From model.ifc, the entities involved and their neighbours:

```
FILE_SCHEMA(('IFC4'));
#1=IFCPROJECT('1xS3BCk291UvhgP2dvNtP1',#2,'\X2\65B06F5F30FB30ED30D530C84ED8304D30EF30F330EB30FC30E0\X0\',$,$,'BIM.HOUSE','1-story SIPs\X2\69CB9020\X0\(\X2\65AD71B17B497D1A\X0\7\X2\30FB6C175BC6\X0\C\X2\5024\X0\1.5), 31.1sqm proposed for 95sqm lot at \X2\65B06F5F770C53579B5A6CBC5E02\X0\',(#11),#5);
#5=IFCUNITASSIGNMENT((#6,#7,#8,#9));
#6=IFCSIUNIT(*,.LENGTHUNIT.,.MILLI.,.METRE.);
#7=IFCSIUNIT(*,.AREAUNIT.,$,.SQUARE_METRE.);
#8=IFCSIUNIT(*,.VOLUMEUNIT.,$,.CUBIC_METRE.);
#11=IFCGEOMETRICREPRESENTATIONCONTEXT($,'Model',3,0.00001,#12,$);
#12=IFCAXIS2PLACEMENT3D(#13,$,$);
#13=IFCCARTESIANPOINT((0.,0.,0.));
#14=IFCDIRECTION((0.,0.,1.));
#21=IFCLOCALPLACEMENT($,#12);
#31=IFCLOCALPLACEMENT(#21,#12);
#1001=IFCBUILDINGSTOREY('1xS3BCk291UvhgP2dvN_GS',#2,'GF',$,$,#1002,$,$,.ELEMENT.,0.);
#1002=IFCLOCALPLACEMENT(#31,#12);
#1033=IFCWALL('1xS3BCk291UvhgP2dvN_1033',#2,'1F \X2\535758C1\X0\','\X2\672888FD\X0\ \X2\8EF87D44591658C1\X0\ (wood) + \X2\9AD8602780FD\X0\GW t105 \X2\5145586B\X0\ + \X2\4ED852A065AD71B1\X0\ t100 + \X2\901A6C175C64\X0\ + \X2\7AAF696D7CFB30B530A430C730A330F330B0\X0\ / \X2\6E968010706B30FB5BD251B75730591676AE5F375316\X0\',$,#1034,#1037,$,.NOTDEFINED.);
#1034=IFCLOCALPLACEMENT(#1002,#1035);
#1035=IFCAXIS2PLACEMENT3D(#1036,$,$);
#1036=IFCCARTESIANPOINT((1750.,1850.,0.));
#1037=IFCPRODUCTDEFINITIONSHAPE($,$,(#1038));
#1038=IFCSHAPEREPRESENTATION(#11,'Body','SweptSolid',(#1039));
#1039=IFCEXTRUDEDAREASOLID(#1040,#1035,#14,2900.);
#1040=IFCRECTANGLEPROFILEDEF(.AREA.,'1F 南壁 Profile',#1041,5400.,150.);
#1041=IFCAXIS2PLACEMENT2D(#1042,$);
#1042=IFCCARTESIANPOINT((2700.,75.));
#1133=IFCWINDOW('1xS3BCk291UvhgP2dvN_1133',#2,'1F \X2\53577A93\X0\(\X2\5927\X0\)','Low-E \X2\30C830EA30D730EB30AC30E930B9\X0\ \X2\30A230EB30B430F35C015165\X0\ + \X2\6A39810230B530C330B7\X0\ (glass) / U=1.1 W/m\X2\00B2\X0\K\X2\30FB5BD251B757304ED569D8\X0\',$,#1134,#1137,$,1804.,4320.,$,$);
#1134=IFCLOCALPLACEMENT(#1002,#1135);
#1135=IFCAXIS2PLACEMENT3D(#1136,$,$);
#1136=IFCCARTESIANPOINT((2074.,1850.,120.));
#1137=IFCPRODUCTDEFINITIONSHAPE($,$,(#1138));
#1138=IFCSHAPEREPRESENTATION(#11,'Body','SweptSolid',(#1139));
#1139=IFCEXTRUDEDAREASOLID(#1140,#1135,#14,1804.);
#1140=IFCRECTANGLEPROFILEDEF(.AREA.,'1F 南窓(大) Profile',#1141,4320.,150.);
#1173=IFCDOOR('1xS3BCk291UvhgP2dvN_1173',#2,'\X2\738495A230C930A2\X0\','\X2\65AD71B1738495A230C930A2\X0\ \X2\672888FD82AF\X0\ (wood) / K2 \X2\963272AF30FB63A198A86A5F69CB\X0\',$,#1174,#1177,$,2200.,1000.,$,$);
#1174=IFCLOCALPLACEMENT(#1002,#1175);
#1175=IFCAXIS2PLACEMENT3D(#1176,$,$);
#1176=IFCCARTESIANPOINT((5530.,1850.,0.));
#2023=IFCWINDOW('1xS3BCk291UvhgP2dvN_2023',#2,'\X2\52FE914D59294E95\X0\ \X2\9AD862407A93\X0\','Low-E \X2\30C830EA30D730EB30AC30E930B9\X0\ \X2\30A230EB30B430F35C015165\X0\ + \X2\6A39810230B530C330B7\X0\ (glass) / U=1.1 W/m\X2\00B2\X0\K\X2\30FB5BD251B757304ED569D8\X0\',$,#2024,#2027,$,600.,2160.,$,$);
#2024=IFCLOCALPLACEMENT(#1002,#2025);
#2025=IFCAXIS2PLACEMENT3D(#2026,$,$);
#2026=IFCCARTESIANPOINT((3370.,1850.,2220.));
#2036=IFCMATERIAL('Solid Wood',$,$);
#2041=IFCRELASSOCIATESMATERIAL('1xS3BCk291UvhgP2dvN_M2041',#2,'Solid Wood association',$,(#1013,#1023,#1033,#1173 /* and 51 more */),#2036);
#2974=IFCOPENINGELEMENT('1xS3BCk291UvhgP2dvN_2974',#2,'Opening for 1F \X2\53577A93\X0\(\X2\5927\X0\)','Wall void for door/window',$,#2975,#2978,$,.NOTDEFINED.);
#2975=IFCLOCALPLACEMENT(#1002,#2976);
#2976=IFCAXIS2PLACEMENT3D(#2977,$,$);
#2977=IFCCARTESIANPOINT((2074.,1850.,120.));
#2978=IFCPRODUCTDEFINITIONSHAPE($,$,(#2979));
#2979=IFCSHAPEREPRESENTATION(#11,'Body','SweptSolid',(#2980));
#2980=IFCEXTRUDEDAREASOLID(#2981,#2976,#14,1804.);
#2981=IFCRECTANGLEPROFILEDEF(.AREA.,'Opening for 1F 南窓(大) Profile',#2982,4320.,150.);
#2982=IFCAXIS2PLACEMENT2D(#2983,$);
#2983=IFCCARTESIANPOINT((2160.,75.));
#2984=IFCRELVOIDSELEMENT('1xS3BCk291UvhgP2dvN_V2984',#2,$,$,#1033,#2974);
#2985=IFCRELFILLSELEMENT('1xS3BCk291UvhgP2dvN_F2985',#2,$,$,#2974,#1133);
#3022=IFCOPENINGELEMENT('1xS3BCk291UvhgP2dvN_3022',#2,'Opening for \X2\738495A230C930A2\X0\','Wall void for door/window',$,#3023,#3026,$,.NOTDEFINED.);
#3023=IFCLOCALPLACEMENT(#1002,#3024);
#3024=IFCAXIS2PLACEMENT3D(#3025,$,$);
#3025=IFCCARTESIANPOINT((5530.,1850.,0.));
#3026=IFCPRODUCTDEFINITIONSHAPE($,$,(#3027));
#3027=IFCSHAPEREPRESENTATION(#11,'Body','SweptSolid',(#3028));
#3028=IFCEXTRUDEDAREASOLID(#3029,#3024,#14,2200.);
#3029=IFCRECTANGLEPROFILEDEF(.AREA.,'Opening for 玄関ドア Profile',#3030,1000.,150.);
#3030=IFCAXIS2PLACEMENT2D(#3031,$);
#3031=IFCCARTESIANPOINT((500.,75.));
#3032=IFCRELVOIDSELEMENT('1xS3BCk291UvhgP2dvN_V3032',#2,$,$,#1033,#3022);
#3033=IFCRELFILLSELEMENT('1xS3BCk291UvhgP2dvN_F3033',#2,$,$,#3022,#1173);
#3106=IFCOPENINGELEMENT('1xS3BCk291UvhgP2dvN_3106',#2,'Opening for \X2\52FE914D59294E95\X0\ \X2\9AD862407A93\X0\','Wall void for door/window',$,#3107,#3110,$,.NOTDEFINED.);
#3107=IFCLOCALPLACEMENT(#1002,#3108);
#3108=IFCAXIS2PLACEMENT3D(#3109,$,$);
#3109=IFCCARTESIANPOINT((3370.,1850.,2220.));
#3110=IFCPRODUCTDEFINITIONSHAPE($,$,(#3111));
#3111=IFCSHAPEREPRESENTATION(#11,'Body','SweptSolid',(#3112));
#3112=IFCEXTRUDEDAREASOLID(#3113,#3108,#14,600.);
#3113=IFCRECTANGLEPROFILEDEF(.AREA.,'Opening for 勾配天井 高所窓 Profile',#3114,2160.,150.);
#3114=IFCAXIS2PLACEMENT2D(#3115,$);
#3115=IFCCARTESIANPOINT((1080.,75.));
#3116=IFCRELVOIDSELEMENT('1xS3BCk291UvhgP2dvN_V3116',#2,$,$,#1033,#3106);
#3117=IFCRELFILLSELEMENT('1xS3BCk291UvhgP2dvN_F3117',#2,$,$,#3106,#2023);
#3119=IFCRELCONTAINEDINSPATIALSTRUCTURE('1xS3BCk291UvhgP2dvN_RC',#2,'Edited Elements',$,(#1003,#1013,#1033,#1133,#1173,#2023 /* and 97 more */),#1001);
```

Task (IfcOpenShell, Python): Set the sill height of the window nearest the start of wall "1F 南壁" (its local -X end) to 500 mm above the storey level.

```python
import numpy as np
import ifcopenshell
import ifcopenshell.api.geometry
import ifcopenshell.geom
import ifcopenshell.util.element
import ifcopenshell.util.placement
import ifcopenshell.util.shape
import ifcopenshell.util.unit

model = ifcopenshell.open("model.ifc")
unit_scale = ifcopenshell.util.unit.calculate_unit_scale(model)

window = model.by_guid("1xS3BCk291UvhgP2dvN_1133")
opening = window.FillsVoids[0].RelatingOpeningElement
storey = ifcopenshell.util.element.get_container(window, ifc_class="IfcBuildingStorey")
level = ifcopenshell.util.placement.get_local_placement(storey.ObjectPlacement)[2, 3]

# The opening's origin need not be at the sill, so measure its lowest point.
shape = ifcopenshell.geom.create_shape(ifcopenshell.geom.settings(), opening)
bottom = ifcopenshell.util.shape.get_shape_bottom_elevation(shape, shape.geometry) / unit_scale
dz = level + 0.5 / unit_scale - bottom

shift = np.array([0.0, 0.0, dz])
# The window is not placed relative to its opening, so move both.
for product in (opening, window):
    matrix = ifcopenshell.util.placement.get_local_placement(product.ObjectPlacement)
    matrix[:3, 3] += shift
    ifcopenshell.api.geometry.edit_object_placement(model, product=product, matrix=matrix, is_si=False)

print(f"moved by {dz * unit_scale:+.3f} m")

model.write("model-out.ifc")
```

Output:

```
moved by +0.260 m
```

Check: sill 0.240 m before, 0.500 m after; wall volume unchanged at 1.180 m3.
